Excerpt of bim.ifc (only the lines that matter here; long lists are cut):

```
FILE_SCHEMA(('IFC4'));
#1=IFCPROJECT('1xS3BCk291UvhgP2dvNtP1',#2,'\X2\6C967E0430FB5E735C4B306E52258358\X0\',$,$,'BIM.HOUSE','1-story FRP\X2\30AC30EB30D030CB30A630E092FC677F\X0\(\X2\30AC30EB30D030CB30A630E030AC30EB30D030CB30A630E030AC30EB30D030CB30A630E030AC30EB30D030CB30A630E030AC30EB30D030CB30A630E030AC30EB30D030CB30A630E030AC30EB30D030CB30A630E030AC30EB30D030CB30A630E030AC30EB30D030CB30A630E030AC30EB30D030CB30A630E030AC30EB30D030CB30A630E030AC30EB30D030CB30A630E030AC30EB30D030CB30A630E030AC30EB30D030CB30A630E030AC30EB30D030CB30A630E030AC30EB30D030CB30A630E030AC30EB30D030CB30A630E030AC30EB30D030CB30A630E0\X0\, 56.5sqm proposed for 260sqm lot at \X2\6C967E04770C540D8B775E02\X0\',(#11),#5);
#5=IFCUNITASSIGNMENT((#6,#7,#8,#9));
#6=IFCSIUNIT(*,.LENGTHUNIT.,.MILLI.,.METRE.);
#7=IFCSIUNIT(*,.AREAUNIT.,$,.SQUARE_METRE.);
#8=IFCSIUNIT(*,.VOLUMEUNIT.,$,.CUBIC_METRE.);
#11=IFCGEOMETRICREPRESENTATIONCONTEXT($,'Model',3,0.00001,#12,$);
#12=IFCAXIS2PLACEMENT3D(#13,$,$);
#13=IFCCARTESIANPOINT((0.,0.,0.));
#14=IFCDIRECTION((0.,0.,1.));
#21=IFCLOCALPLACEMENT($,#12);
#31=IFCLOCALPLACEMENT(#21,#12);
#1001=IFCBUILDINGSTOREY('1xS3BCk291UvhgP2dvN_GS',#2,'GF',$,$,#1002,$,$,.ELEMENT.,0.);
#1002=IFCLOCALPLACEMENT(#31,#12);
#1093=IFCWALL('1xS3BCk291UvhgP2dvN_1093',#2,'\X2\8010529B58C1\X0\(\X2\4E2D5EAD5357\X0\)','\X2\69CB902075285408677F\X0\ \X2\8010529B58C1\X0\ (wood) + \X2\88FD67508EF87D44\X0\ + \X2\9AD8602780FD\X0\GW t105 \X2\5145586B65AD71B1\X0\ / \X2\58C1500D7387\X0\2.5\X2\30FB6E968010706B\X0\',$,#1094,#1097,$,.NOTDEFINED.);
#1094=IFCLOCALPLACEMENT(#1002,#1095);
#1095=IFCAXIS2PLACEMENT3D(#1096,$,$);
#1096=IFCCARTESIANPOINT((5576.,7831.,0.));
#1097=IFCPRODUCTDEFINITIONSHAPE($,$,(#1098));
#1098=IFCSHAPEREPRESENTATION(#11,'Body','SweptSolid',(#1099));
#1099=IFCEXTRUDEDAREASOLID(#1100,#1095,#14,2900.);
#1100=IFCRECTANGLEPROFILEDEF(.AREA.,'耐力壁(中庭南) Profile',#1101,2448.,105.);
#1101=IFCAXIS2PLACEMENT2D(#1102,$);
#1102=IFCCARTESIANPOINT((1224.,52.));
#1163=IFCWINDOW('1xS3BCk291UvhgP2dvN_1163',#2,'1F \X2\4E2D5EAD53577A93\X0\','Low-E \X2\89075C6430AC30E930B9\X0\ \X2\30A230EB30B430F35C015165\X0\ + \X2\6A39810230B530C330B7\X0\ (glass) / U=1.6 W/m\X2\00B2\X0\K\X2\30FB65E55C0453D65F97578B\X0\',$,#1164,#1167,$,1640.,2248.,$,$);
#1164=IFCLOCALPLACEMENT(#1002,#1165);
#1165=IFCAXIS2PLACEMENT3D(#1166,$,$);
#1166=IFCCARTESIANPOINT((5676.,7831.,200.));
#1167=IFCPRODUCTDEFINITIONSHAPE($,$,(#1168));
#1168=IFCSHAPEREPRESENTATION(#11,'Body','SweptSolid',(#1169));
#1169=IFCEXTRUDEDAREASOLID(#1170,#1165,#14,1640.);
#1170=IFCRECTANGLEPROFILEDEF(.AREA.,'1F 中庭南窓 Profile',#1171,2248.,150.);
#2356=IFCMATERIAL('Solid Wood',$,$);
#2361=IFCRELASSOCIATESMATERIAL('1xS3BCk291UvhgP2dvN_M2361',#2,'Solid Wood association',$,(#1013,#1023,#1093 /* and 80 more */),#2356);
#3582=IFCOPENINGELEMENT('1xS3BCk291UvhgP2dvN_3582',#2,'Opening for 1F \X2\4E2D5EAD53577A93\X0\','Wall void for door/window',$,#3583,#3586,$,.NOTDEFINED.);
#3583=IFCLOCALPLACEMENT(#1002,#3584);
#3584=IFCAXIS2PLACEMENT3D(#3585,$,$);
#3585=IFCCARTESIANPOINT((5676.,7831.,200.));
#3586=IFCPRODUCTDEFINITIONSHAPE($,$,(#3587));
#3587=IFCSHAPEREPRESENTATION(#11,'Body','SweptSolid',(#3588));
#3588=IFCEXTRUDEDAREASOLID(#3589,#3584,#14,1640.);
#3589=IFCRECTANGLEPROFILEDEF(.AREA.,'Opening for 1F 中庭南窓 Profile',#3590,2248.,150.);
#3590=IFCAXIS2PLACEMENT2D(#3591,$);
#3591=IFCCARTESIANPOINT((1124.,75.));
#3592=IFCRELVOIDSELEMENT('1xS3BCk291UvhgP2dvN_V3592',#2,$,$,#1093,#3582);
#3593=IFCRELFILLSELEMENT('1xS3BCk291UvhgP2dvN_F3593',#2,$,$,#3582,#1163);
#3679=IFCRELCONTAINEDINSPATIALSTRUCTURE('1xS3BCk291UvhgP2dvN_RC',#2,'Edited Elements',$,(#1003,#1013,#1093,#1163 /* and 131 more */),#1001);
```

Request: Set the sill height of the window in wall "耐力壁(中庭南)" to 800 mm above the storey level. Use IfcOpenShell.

```python
import numpy as np
import ifcopenshell
import ifcopenshell.api.geometry
import ifcopenshell.geom
import ifcopenshell.util.element
import ifcopenshell.util.placement
import ifcopenshell.util.shape
import ifcopenshell.util.unit

model = ifcopenshell.open("bim.ifc")
unit_scale = ifcopenshell.util.unit.calculate_unit_scale(model)

window = model.by_guid("1xS3BCk291UvhgP2dvN_1163")
opening = window.FillsVoids[0].RelatingOpeningElement
storey = ifcopenshell.util.element.get_container(window, ifc_class="IfcBuildingStorey")
level = ifcopenshell.util.placement.get_local_placement(storey.ObjectPlacement)[2, 3]

# The opening's origin need not be at the sill, so measure its lowest point.
shape = ifcopenshell.geom.create_shape(ifcopenshell.geom.settings(), opening)
bottom = ifcopenshell.util.shape.get_shape_bottom_elevation(shape, shape.geometry) / unit_scale
dz = level + 800.0 - bottom

shift = np.array([0.0, 0.0, dz])
# The window is not placed relative to its opening, so move both.
for product in (opening, window):
    matrix = ifcopenshell.util.placement.get_local_placement(product.ObjectPlacement)
    matrix[:3, 3] += shift
    ifcopenshell.api.geometry.edit_object_placement(model, product=product, matrix=matrix, is_si=False)

print(f"moved by {dz * unit_scale:+.3f} m")

model.write("bim_edited.ifc")
```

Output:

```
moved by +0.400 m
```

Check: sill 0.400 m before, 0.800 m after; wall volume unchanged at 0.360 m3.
